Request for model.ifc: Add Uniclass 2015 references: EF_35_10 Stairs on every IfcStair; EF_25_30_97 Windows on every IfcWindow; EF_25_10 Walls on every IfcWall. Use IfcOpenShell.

First a look at what the model holds.

```python
import ifcopenshell

model = ifcopenshell.open("model.ifc")
print(model.schema)
print("classifications:", [c.Name for c in model.by_type("IfcClassification")])
for ifc_class in ("IfcDoor", "IfcRoof", "IfcStair", "IfcWall", "IfcWindow"):
    print(ifc_class, len(model.by_type(ifc_class)))
```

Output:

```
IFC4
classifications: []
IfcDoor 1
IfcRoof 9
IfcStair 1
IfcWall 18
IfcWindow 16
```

```python
import ifcopenshell
import ifcopenshell.api.classification

model = ifcopenshell.open("model.ifc")

system = ifcopenshell.api.classification.add_classification(model, classification="Uniclass 2015")

codes = {
    "IfcStair": ("EF_35_10", "Stairs"),
    "IfcWindow": ("EF_25_30_97", "Windows"),
    "IfcWall": ("EF_25_10", "Walls"),
}
for ifc_class, (code, name) in codes.items():
    products = model.by_type(ifc_class)
    ifcopenshell.api.classification.add_reference(
        model, products=products, classification=system, identification=code, name=name
    )
    print(code, len(products))

model.write("model_updated.ifc")
```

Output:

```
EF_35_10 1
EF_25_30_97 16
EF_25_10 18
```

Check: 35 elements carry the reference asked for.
